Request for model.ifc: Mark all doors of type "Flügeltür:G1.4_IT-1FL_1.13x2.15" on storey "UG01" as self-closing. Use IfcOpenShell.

First a look at what the model holds.

```python
import ifcopenshell
import ifcopenshell.util.element

model = ifcopenshell.open("model.ifc")
print(model.schema)
storey = next(s for s in model.by_type("IfcBuildingStorey") if s.Name == "UG01")
doors = [e for e in ifcopenshell.util.element.get_decomposition(storey) if e.is_a("IfcDoor")]
seen = {}
for e in doors:
    element_type = ifcopenshell.util.element.get_type(e)
    key = (element_type.Name if element_type != e and element_type else None, ifcopenshell.util.element.get_pset(e, "Pset_DoorCommon", "SelfClosing"))
    seen[key] = seen.get(key, 0) + 1
for (name, value), count in sorted(seen.items(), key=str):
    print(count, "x", name, "|", value)
```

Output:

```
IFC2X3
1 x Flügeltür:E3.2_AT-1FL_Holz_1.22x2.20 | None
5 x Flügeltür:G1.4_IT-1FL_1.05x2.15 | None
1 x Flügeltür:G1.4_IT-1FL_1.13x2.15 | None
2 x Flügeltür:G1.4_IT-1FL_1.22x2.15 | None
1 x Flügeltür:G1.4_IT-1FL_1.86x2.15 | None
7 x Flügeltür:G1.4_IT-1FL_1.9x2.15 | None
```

```python
import ifcopenshell
import ifcopenshell.api.pset
import ifcopenshell.util.element

model = ifcopenshell.open("model.ifc")

storey = next(s for s in model.by_type("IfcBuildingStorey") if s.Name == "UG01")
doors = [e for e in ifcopenshell.util.element.get_decomposition(storey) if e.is_a("IfcDoor")]

count = 0
for e in doors:
    element_type = ifcopenshell.util.element.get_type(e)
    if element_type in (None, e) or element_type.Name != "Flügeltür:G1.4_IT-1FL_1.13x2.15":
        continue
    # add_pset returns the element's existing set when there is one.
    pset = ifcopenshell.api.pset.add_pset(model, product=e, name="Pset_DoorCommon")
    ifcopenshell.api.pset.edit_pset(model, pset=pset, properties={"SelfClosing": True})
    count += 1

print(count, "doors updated")

model.write("model_v2.ifc")
```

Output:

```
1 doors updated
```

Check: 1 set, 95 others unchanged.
